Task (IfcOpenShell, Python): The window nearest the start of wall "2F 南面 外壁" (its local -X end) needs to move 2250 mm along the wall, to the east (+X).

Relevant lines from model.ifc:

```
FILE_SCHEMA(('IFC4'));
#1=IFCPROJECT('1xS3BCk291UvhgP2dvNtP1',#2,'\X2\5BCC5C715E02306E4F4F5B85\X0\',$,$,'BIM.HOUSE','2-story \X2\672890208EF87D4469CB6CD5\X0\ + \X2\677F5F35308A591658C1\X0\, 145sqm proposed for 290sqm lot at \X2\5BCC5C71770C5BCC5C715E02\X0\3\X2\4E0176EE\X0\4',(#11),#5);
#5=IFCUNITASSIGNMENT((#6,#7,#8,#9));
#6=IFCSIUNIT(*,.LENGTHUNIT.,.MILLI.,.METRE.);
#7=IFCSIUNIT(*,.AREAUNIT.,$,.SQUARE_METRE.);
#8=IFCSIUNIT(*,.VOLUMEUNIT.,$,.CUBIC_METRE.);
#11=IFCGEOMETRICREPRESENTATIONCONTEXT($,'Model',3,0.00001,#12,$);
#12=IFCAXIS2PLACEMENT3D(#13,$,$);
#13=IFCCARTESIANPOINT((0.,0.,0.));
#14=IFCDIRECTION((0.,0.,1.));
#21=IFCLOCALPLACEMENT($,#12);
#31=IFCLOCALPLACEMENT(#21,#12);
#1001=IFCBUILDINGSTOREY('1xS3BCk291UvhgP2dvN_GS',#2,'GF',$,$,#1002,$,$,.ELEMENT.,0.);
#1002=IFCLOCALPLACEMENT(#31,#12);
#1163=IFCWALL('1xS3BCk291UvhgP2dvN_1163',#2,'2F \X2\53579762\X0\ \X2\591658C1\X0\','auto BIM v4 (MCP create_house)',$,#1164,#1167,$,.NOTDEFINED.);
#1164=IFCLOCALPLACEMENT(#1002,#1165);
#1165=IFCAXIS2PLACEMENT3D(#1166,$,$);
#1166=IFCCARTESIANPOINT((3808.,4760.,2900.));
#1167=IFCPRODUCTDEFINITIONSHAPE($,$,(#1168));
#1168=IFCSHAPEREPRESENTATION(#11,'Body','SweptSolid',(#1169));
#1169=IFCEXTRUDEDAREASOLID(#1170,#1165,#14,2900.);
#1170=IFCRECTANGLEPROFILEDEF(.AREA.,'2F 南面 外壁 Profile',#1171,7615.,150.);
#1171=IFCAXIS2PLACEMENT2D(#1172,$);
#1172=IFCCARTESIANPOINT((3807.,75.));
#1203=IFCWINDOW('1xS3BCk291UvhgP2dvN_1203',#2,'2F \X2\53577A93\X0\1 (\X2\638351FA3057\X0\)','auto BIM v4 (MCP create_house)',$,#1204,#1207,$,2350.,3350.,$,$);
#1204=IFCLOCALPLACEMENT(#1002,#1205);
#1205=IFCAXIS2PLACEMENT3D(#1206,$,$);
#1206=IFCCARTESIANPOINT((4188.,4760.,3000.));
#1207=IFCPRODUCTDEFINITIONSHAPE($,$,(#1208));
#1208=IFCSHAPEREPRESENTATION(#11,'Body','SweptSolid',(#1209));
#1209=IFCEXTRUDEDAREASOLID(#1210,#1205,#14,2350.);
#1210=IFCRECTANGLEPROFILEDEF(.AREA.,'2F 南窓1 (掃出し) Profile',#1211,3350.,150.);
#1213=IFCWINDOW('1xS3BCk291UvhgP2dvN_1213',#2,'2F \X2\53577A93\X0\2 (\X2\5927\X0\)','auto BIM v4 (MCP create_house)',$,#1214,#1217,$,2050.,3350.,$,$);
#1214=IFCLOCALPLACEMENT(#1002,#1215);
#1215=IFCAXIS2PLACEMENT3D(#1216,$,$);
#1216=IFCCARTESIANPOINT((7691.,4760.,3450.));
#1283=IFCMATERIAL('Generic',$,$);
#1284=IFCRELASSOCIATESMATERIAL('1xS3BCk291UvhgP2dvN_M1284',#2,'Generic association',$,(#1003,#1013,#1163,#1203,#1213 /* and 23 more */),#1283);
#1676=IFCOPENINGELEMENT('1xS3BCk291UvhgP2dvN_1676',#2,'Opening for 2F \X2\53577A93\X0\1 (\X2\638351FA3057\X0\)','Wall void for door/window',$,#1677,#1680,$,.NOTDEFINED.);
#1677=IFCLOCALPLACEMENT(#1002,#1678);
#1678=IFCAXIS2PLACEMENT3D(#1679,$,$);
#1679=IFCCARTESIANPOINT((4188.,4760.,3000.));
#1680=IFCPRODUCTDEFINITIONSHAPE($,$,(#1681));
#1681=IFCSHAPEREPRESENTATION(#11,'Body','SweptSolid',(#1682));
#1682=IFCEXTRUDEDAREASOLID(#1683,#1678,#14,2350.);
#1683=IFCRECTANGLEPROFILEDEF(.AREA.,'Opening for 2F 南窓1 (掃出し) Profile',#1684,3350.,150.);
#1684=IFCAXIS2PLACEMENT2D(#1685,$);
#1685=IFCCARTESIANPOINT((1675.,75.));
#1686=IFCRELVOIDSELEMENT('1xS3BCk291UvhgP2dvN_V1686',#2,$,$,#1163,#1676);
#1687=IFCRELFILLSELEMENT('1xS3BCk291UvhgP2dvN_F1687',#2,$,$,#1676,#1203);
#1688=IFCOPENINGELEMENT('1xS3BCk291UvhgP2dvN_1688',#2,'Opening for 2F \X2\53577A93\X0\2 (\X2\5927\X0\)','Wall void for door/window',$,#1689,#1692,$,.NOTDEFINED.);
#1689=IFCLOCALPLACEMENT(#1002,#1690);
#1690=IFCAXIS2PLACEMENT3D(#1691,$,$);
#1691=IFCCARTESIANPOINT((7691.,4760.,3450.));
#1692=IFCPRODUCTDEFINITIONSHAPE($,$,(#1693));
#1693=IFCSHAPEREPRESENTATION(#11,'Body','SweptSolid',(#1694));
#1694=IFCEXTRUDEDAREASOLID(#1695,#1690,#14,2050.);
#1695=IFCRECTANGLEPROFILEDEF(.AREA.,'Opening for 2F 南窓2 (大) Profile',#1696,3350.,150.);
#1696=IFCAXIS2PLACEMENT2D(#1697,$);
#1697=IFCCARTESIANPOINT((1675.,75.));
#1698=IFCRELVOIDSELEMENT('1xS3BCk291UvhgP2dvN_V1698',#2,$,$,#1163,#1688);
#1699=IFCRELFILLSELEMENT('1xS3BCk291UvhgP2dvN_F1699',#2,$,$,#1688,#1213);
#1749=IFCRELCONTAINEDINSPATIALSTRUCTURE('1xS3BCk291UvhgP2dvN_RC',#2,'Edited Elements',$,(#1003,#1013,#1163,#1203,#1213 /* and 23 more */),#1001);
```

```python
import ifcopenshell
import ifcopenshell.api.geometry
import ifcopenshell.util.placement
import ifcopenshell.util.unit

model = ifcopenshell.open("model.ifc")
unit_scale = ifcopenshell.util.unit.calculate_unit_scale(model)

window = model.by_guid("1xS3BCk291UvhgP2dvN_1203")
opening = window.FillsVoids[0].RelatingOpeningElement
wall = opening.VoidsElements[0].RelatingBuildingElement

wall_matrix = ifcopenshell.util.placement.get_local_placement(wall.ObjectPlacement)
shift = wall_matrix[:3, 0] * 2.25 / unit_scale
before = ifcopenshell.util.placement.get_local_placement(window.ObjectPlacement)[:3, 3].copy()

# The window is not placed relative to its opening, so move both.
for product in (opening, window):
    matrix = ifcopenshell.util.placement.get_local_placement(product.ObjectPlacement)
    matrix[:3, 3] += shift
    ifcopenshell.api.geometry.edit_object_placement(model, product=product, matrix=matrix, is_si=False)

after = ifcopenshell.util.placement.get_local_placement(window.ObjectPlacement)[:3, 3]
print("window moved by", (after - before).round(3) + 0.0)

model.write("model_rev.ifc")
```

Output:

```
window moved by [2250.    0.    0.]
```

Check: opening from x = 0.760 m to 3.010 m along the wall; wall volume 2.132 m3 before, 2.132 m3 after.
